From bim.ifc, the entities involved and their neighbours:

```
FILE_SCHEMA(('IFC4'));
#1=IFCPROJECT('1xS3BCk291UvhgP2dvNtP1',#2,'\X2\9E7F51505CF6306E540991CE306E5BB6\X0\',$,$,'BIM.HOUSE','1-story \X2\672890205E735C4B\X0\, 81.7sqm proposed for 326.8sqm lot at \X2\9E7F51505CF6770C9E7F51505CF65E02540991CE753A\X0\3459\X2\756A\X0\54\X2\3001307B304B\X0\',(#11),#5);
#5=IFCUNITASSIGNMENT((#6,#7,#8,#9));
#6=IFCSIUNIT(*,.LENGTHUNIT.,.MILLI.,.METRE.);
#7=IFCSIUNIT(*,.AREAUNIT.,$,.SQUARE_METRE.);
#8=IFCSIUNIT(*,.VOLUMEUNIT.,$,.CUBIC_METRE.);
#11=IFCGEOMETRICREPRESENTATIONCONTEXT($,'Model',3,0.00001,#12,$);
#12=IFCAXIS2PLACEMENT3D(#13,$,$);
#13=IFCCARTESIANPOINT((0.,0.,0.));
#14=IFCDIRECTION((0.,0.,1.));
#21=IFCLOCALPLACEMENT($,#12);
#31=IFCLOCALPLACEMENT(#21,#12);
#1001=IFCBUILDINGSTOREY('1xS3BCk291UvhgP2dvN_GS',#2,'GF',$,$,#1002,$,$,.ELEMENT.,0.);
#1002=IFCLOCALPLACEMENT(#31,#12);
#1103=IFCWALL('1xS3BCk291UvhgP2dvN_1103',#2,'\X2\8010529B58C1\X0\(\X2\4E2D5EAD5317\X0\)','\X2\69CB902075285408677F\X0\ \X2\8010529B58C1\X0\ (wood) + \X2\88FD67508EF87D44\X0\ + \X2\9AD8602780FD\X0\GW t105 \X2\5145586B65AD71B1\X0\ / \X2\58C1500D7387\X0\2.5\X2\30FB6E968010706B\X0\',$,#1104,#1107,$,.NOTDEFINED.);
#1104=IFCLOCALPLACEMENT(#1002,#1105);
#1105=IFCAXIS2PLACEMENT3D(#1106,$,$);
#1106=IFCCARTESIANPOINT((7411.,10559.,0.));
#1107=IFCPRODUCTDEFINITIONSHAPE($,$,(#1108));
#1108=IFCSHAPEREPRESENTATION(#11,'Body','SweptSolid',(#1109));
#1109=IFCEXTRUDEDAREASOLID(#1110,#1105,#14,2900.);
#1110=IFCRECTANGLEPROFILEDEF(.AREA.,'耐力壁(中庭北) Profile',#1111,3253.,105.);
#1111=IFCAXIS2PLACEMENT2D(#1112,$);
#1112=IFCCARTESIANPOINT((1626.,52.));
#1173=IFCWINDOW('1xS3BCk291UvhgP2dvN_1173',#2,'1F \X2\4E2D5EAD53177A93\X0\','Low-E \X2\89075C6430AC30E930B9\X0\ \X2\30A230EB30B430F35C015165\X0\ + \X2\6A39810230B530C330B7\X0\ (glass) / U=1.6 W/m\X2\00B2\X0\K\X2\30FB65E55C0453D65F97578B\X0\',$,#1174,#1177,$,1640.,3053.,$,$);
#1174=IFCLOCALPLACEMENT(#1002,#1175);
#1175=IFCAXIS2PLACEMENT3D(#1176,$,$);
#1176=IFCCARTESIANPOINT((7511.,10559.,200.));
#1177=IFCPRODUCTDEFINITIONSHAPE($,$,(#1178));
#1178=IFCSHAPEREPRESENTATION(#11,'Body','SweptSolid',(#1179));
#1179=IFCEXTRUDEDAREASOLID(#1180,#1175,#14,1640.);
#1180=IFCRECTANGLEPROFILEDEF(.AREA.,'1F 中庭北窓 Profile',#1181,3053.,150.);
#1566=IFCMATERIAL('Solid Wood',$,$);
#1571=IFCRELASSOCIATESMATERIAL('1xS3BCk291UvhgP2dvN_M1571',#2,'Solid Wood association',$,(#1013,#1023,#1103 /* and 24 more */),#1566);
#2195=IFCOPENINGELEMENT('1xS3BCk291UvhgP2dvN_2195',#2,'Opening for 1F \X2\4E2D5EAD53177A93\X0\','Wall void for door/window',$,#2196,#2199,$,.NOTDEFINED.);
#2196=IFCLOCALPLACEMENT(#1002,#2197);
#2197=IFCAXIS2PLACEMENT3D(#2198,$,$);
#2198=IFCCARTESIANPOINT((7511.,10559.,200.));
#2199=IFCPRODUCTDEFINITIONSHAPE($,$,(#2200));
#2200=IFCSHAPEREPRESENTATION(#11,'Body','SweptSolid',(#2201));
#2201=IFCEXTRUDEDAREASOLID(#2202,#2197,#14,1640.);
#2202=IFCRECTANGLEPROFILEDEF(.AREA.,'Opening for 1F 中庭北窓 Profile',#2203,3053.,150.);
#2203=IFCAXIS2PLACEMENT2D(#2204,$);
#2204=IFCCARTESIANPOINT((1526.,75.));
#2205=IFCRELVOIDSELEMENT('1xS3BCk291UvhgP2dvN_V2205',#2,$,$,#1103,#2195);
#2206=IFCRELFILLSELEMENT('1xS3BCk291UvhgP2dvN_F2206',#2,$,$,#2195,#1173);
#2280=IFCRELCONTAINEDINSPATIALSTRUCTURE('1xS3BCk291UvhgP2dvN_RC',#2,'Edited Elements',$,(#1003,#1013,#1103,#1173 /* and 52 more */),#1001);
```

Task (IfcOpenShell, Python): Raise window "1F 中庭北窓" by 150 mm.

```python
import numpy as np
import ifcopenshell
import ifcopenshell.api.geometry
import ifcopenshell.util.placement
import ifcopenshell.util.unit

model = ifcopenshell.open("bim.ifc")
unit_scale = ifcopenshell.util.unit.calculate_unit_scale(model)

window = model.by_guid("1xS3BCk291UvhgP2dvN_1173")
opening = window.FillsVoids[0].RelatingOpeningElement
dz = 150.0

shift = np.array([0.0, 0.0, dz])
# The window is not placed relative to its opening, so move both.
for product in (opening, window):
    matrix = ifcopenshell.util.placement.get_local_placement(product.ObjectPlacement)
    matrix[:3, 3] += shift
    ifcopenshell.api.geometry.edit_object_placement(model, product=product, matrix=matrix, is_si=False)

print(f"moved by {dz * unit_scale:+.3f} m")

model.write("bim-out.ifc")
```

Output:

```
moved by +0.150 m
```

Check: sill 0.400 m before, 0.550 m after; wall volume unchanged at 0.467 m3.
